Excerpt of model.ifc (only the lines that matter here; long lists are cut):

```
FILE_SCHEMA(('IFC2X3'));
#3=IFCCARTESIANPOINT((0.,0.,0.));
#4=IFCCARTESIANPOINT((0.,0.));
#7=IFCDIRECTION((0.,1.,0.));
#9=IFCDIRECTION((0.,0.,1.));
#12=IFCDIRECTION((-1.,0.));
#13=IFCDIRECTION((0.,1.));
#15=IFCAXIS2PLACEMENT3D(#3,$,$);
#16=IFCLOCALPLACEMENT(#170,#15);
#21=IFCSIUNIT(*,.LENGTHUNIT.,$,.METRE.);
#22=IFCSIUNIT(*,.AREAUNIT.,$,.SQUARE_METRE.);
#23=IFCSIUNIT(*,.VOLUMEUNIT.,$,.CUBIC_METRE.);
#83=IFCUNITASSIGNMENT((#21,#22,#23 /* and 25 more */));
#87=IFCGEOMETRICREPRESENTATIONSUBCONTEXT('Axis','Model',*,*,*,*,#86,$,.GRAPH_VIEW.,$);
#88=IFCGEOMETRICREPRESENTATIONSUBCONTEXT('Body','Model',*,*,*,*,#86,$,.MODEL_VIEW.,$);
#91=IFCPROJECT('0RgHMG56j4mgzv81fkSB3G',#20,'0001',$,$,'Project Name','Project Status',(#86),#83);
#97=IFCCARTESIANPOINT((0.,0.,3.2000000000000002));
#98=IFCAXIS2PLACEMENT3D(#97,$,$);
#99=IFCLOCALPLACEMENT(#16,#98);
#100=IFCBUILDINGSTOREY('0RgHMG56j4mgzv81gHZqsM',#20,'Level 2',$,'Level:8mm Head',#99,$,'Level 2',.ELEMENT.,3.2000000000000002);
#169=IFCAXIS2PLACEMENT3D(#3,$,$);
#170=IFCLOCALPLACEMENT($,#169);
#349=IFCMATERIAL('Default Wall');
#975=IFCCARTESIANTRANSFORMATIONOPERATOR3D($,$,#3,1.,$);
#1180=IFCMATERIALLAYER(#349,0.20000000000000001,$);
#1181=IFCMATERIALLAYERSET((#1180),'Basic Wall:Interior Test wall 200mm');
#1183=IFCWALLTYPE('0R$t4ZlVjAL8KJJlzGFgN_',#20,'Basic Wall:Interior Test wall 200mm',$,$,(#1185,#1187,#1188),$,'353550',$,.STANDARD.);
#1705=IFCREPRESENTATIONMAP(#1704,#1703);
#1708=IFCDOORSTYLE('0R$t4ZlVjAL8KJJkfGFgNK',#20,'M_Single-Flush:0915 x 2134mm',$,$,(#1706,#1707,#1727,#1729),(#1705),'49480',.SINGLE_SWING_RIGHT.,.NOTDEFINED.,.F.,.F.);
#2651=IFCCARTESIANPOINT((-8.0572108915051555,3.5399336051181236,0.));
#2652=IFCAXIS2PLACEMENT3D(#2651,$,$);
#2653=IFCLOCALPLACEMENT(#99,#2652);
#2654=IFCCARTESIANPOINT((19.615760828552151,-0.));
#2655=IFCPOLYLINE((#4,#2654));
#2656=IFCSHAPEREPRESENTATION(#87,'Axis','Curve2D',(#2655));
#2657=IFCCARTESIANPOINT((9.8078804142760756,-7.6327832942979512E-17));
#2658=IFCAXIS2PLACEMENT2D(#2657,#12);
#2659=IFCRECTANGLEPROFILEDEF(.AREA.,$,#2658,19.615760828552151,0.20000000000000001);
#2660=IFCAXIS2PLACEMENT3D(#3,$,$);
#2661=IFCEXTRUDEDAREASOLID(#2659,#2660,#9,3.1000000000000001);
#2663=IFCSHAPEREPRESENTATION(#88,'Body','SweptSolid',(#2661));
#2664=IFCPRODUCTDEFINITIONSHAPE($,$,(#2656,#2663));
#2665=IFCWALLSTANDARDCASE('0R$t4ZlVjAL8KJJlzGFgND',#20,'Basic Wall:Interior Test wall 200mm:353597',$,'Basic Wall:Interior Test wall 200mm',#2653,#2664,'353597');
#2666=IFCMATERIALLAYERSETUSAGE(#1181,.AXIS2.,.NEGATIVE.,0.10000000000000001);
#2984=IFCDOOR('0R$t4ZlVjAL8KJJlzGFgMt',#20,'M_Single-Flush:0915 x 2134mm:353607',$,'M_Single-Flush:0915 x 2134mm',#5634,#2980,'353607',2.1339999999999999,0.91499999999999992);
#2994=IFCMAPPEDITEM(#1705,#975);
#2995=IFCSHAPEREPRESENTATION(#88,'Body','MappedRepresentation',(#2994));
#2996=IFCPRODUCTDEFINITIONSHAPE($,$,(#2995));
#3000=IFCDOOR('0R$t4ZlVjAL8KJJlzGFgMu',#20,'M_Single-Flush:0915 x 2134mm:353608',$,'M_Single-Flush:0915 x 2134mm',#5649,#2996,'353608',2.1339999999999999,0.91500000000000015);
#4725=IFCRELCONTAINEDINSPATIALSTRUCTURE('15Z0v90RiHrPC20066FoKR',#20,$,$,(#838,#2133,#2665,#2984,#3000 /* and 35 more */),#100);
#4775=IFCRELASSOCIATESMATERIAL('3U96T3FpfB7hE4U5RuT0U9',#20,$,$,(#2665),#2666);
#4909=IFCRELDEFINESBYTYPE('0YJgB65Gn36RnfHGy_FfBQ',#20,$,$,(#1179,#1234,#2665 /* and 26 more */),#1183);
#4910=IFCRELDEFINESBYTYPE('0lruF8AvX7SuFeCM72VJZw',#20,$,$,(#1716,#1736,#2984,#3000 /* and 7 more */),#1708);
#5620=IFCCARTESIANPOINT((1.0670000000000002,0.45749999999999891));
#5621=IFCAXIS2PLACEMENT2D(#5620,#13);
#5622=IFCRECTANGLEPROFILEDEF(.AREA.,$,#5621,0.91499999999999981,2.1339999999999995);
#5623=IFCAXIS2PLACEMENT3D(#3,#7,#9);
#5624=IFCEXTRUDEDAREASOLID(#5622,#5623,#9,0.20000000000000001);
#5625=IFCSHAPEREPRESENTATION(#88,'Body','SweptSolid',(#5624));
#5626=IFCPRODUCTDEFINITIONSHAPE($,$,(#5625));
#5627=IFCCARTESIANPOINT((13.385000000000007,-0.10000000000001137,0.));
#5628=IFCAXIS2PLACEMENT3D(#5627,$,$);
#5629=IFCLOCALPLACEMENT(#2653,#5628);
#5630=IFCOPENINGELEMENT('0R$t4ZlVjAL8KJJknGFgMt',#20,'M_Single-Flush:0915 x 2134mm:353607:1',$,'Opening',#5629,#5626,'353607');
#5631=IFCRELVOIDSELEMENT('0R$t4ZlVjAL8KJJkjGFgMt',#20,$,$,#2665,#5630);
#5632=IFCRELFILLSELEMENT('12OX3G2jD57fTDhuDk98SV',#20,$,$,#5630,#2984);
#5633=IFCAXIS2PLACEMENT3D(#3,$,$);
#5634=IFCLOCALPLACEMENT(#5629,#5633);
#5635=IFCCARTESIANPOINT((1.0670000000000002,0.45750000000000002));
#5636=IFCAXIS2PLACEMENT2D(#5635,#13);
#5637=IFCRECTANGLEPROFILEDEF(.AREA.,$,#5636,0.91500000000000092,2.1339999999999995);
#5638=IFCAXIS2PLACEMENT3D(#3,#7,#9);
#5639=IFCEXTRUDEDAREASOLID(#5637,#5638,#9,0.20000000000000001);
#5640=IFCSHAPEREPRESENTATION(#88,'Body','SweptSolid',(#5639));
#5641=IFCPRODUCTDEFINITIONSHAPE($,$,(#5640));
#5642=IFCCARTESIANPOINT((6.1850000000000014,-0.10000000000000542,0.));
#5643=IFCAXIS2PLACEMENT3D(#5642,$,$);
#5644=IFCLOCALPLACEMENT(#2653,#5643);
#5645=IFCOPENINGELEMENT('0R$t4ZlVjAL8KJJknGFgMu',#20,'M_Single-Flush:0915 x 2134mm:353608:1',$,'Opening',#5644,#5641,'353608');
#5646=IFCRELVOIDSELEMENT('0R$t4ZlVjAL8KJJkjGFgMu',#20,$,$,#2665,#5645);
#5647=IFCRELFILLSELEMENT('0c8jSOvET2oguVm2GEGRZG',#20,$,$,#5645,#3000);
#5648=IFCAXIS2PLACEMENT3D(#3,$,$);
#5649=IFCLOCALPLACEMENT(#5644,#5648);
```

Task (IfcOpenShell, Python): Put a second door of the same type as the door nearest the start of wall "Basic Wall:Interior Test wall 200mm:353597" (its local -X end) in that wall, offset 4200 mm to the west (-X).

```python
import ifcopenshell
import ifcopenshell.api.feature
import ifcopenshell.api.geometry
import ifcopenshell.api.root
import ifcopenshell.geom
import ifcopenshell.util.element
import ifcopenshell.util.placement
import ifcopenshell.util.shape
import ifcopenshell.util.unit

model = ifcopenshell.open("model.ifc")
unit_scale = ifcopenshell.util.unit.calculate_unit_scale(model)
settings = ifcopenshell.geom.settings()


def volume(element):
    """Net volume in cubic metres, openings subtracted."""
    shape = ifcopenshell.geom.create_shape(settings, element)
    return ifcopenshell.util.shape.get_volume(shape.geometry)


def reuse_history(source, copy):
    """copy_class also copies each property set's owner history, people and application; keep the originals."""
    for rel in copy.IsDefinedBy:
        if rel.is_a("IfcRelDefinesByProperties") and (history := rel.RelatingPropertyDefinition.OwnerHistory):
            rel.RelatingPropertyDefinition.OwnerHistory = source.OwnerHistory
            ifcopenshell.util.element.remove_deep2(model, history)


door = model.by_guid("0R$t4ZlVjAL8KJJlzGFgMu")
opening = door.FillsVoids[0].RelatingOpeningElement
wall = opening.VoidsElements[0].RelatingBuildingElement
before = volume(wall)
shift = ifcopenshell.util.placement.get_local_placement(wall.ObjectPlacement)[:3, 0] * -4.2 / unit_scale

# copy_class copies the void relationship, type, container and properties, but no geometry.
new_opening = ifcopenshell.api.root.copy_class(model, product=opening)
new_opening.Representation = ifcopenshell.util.element.copy_deep(
    model, opening.Representation, exclude=["IfcGeometricRepresentationContext", "IfcRepresentationMap"]
)
new_opening.Name = "M_Single-Flush:0915 x 2134mm"
new_opening.Tag = None
new_door = ifcopenshell.api.root.copy_class(model, product=door)
new_door.Representation = ifcopenshell.util.element.copy_deep(
    model, door.Representation, exclude=["IfcGeometricRepresentationContext", "IfcRepresentationMap"]
)
new_door.Name = "M_Single-Flush:0915 x 2134mm"
new_door.Tag = None
reuse_history(door, new_door)
fills = ifcopenshell.api.feature.add_filling(model, opening=new_opening, element=new_door)
fills.OwnerHistory = new_door.OwnerHistory  # required in IFC2X3

for old, new in ((opening, new_opening), (door, new_door)):
    matrix = ifcopenshell.util.placement.get_local_placement(old.ObjectPlacement)
    matrix[:3, 3] += shift
    ifcopenshell.api.geometry.edit_object_placement(model, product=new, matrix=matrix, is_si=False)

after = volume(wall)

print(f"wall volume {before:.3f} -> {after:.3f} m3")

model.write("model_updated.ifc")
```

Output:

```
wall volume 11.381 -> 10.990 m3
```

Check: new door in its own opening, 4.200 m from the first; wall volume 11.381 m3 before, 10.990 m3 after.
